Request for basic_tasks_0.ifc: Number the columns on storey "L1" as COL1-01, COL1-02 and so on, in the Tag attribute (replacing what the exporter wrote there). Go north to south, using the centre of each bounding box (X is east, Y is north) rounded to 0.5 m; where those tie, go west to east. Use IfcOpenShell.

First a look at what the model holds.

```python
import ifcopenshell
import ifcopenshell.util.element
import ifcopenshell.util.placement

model = ifcopenshell.open("basic_tasks_0.ifc")
print(model.schema)
storey = next(s for s in model.by_type("IfcBuildingStorey") if s.Name == "L1")
columns = [e for e in ifcopenshell.util.element.get_decomposition(storey) if e.is_a("IfcColumn")]
for e in sorted(columns, key=lambda e: e.id()):
    origin = ifcopenshell.util.placement.get_local_placement(e.ObjectPlacement)[:3, 3]
    print(e.id(), e.Tag, e.Name, origin.round(2) + 0.0, sep=" | ")
```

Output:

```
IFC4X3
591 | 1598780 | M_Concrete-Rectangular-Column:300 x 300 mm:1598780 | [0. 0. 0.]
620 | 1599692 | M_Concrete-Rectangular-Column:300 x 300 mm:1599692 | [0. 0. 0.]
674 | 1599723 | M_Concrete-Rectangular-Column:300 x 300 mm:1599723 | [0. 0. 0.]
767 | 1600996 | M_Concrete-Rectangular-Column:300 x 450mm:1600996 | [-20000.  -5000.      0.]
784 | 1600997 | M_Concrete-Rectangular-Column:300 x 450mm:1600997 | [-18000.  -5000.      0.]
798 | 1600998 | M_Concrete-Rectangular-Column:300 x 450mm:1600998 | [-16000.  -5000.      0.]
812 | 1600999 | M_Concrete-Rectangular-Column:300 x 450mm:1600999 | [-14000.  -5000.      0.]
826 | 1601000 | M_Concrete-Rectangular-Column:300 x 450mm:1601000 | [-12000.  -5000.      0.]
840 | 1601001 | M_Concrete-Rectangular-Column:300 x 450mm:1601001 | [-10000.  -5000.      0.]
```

```python
import ifcopenshell
import ifcopenshell.geom
import ifcopenshell.util.element
import ifcopenshell.util.shape

model = ifcopenshell.open("basic_tasks_0.ifc")
settings = ifcopenshell.geom.settings()
settings.set("use-world-coords", True)


def centre(element):
    shape = ifcopenshell.geom.create_shape(settings, element)
    return ifcopenshell.util.shape.get_bbox_centroid(shape.geometry)


storey = next(s for s in model.by_type("IfcBuildingStorey") if s.Name == "L1")
columns = [e for e in ifcopenshell.util.element.get_decomposition(storey) if e.is_a("IfcColumn")]

# Insertion points can sit at a corner or the storey origin, so sort by the geometry (in metres).
centres = {e: centre(e) for e in columns}
columns.sort(key=lambda e: (-round(centres[e][1] / 0.5), centres[e][0]))

for i, e in enumerate(columns, start=1):
    number = f"COL1-{i:02d}"
    e.Tag = number
    print(e.id(), number)

model.write("basic_tasks_0_v2.ifc")
```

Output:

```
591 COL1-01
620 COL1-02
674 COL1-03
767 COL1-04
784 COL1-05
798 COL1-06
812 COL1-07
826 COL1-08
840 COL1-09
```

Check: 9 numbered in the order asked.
